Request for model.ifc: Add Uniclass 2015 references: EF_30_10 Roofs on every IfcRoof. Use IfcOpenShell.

First a look at what the model holds.

```python
import ifcopenshell

model = ifcopenshell.open("model.ifc")
print(model.schema)
print("classifications:", [c.Name for c in model.by_type("IfcClassification")])
for ifc_class in ("IfcDoor", "IfcRoof", "IfcStair", "IfcWall", "IfcWindow"):
    print(ifc_class, len(model.by_type(ifc_class)))
```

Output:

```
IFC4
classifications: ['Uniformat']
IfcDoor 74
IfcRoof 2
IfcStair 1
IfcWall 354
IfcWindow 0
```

```python
import ifcopenshell
import ifcopenshell.api.classification

model = ifcopenshell.open("model.ifc")

system = ifcopenshell.api.classification.add_classification(model, classification="Uniclass 2015")

codes = {
    "IfcRoof": ("EF_30_10", "Roofs"),
}
for ifc_class, (code, name) in codes.items():
    products = model.by_type(ifc_class)
    ifcopenshell.api.classification.add_reference(
        model, products=products, classification=system, identification=code, name=name
    )
    print(code, len(products))

model.write("model-out.ifc")
```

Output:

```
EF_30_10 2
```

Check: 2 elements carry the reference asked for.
